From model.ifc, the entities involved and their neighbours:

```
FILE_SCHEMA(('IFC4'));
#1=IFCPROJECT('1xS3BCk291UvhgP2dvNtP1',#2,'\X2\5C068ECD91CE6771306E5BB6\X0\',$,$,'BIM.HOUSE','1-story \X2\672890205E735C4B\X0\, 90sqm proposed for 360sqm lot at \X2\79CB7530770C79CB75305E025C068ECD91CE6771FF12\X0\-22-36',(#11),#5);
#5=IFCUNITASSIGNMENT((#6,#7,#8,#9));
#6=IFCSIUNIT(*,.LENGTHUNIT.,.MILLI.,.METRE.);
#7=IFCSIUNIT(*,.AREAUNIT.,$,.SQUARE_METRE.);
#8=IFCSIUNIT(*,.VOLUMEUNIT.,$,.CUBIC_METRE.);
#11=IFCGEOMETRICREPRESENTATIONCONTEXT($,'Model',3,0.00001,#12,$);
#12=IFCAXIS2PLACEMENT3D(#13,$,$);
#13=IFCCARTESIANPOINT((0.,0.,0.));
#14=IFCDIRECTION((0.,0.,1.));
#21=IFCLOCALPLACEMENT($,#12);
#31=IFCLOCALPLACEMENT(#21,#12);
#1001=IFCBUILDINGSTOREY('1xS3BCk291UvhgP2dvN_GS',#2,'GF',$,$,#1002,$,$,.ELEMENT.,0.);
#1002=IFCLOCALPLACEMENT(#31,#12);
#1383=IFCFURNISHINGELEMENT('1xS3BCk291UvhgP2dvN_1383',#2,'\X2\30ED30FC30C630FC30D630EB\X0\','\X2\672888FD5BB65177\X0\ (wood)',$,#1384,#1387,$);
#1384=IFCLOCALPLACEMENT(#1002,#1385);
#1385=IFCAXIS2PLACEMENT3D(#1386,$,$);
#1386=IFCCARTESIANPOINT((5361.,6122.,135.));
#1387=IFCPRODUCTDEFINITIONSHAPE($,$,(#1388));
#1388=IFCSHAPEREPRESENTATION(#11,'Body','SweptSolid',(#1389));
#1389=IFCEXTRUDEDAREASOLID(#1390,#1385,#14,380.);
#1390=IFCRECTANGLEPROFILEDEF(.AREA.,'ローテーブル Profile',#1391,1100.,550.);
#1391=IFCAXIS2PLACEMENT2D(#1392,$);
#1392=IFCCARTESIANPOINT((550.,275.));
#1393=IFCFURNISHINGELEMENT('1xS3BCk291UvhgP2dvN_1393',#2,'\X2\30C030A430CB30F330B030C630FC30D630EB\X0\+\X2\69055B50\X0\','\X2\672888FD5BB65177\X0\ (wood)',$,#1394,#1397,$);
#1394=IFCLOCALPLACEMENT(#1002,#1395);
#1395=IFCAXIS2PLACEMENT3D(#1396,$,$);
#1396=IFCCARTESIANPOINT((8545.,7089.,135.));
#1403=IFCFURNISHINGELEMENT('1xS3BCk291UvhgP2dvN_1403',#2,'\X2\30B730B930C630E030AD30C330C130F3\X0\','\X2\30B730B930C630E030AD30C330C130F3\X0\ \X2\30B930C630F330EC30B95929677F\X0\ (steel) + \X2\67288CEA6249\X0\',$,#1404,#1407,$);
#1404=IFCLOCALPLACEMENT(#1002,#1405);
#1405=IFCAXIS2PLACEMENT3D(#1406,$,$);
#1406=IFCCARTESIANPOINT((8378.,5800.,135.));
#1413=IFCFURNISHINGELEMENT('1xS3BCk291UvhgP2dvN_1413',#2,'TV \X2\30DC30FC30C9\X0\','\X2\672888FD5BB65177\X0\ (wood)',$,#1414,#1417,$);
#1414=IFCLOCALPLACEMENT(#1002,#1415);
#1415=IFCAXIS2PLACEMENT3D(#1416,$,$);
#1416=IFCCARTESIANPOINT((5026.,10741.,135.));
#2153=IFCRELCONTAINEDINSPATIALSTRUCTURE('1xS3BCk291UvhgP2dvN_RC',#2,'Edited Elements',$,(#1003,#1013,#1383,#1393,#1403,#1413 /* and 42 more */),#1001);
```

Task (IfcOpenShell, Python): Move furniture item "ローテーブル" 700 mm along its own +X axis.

```python
import ifcopenshell
import ifcopenshell.api.geometry
import ifcopenshell.util.placement
import ifcopenshell.util.unit

model = ifcopenshell.open("model.ifc")
unit_scale = ifcopenshell.util.unit.calculate_unit_scale(model)

item = model.by_guid("1xS3BCk291UvhgP2dvN_1383")
matrix = ifcopenshell.util.placement.get_local_placement(item.ObjectPlacement)
matrix[:3, 3] += matrix[:3, 0] * 0.7 / unit_scale
ifcopenshell.api.geometry.edit_object_placement(model, product=item, matrix=matrix, is_si=False)

print(ifcopenshell.util.placement.get_local_placement(item.ObjectPlacement).round(3) + 0.0)

model.write("model-out.ifc")
```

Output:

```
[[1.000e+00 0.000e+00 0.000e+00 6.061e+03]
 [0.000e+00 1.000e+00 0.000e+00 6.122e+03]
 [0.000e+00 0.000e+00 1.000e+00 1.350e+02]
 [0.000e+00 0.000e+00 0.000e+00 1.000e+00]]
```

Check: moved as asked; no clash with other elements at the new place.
